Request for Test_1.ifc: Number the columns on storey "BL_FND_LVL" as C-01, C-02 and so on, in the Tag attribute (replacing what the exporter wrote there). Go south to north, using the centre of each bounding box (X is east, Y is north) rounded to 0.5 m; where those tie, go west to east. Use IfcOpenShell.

First a look at what the model holds.

```python
import ifcopenshell
import ifcopenshell.util.element
import ifcopenshell.util.placement

model = ifcopenshell.open("Test_1.ifc")
print(model.schema)
storey = next(s for s in model.by_type("IfcBuildingStorey") if s.Name == "BL_FND_LVL")
columns = [e for e in ifcopenshell.util.element.get_decomposition(storey) if e.is_a("IfcColumn")]
for e in sorted(columns, key=lambda e: e.id()):
    origin = ifcopenshell.util.placement.get_local_placement(e.ObjectPlacement)[:3, 3]
    print(e.id(), e.Tag, e.Name, origin.round(2) + 0.0, sep=" | ")
```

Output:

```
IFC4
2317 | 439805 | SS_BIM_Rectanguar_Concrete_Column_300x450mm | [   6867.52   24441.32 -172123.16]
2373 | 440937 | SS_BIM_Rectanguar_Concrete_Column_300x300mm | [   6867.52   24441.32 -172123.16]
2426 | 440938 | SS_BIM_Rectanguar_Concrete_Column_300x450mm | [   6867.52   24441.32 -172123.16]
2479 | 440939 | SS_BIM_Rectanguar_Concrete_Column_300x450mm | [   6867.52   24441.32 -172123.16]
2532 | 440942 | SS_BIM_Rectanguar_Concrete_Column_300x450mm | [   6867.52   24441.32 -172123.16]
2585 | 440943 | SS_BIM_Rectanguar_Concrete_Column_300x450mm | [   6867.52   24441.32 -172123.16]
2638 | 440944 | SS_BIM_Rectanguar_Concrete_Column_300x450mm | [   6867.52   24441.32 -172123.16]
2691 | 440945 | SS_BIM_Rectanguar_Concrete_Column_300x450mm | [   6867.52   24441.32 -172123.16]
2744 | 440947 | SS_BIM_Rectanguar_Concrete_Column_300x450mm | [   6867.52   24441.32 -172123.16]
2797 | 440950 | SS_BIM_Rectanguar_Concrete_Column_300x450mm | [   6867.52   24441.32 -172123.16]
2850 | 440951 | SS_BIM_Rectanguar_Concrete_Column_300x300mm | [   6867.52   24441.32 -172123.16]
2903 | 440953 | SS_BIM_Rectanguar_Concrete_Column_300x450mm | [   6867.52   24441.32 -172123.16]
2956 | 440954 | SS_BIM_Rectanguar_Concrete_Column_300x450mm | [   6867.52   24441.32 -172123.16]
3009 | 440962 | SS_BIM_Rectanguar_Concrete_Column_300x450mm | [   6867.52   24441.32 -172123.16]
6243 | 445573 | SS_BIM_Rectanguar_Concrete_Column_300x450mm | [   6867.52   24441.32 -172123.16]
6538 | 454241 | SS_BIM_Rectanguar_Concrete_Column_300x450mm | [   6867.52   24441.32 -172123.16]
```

```python
import ifcopenshell
import ifcopenshell.geom
import ifcopenshell.util.element
import ifcopenshell.util.shape

model = ifcopenshell.open("Test_1.ifc")
settings = ifcopenshell.geom.settings()
settings.set("use-world-coords", True)


def centre(element):
    shape = ifcopenshell.geom.create_shape(settings, element)
    return ifcopenshell.util.shape.get_bbox_centroid(shape.geometry)


storey = next(s for s in model.by_type("IfcBuildingStorey") if s.Name == "BL_FND_LVL")
columns = [e for e in ifcopenshell.util.element.get_decomposition(storey) if e.is_a("IfcColumn")]

# Insertion points can sit at a corner or the storey origin, so sort by the geometry (in metres).
centres = {e: centre(e) for e in columns}
columns.sort(key=lambda e: (round(centres[e][1] / 0.5), centres[e][0]))

for i, e in enumerate(columns, start=1):
    number = f"C-{i:02d}"
    e.Tag = number
    print(e.id(), number)

model.write("Test_1_rev.ifc")
```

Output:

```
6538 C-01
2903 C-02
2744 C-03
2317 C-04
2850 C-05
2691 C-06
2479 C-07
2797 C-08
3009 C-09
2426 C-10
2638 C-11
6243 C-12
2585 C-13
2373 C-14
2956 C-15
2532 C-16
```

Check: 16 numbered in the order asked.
